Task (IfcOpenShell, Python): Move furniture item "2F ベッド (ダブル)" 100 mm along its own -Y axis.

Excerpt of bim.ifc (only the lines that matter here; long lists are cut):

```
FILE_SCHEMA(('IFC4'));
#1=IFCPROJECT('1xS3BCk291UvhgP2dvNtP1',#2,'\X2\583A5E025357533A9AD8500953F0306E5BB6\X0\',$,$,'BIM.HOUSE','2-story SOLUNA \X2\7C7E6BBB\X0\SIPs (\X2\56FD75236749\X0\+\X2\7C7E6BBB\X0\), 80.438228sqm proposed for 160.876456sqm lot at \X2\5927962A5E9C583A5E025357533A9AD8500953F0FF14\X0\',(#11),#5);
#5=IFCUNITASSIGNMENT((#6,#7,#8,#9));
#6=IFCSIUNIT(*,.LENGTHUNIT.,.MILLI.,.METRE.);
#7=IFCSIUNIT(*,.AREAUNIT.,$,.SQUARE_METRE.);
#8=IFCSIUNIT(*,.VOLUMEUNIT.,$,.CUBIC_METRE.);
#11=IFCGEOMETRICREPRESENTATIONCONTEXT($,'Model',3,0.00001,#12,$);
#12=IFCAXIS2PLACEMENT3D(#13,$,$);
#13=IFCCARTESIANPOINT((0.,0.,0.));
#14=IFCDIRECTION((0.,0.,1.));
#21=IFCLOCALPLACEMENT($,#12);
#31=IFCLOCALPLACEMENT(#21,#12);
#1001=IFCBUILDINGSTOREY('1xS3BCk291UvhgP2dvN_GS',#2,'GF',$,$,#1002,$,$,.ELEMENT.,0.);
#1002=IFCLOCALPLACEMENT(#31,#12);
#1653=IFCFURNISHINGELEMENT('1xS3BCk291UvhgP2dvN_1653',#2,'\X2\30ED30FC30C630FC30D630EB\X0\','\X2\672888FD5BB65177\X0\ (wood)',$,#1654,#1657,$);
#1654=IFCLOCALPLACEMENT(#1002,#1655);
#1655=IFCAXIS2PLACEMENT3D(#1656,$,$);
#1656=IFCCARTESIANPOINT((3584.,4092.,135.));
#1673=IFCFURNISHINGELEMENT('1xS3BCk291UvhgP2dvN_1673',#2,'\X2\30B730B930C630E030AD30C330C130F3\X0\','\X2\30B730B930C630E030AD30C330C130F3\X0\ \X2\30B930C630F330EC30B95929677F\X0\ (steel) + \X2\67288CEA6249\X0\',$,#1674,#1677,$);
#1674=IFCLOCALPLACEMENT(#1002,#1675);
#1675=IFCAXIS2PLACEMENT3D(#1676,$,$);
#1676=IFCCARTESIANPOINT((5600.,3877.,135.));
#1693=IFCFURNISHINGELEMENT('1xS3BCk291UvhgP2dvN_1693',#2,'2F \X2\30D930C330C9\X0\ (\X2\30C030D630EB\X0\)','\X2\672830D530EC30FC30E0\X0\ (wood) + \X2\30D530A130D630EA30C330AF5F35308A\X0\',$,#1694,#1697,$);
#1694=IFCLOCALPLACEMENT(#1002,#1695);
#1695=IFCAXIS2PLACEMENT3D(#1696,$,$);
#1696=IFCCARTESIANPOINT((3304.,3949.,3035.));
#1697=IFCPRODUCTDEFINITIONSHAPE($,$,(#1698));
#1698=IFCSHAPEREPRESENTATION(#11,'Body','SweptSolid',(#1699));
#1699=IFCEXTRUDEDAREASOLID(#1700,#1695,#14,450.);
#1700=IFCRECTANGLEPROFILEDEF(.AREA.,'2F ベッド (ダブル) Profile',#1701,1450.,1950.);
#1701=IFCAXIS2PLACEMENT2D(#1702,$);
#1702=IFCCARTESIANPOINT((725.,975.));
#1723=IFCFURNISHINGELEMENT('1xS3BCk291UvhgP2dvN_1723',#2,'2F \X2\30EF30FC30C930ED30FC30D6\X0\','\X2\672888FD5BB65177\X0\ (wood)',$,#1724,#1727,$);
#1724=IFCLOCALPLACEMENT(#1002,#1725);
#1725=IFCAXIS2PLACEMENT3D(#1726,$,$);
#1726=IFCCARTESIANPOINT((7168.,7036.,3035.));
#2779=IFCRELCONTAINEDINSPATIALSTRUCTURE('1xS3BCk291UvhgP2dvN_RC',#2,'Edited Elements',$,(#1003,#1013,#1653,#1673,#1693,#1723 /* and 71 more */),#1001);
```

```python
import ifcopenshell
import ifcopenshell.api.geometry
import ifcopenshell.util.placement

model = ifcopenshell.open("bim.ifc")

item = model.by_guid("1xS3BCk291UvhgP2dvN_1693")
matrix = ifcopenshell.util.placement.get_local_placement(item.ObjectPlacement)
matrix[:3, 3] -= matrix[:3, 1] * 100.0
ifcopenshell.api.geometry.edit_object_placement(model, product=item, matrix=matrix, is_si=False)

print(ifcopenshell.util.placement.get_local_placement(item.ObjectPlacement).round(3) + 0.0)

model.write("bim_updated.ifc")
```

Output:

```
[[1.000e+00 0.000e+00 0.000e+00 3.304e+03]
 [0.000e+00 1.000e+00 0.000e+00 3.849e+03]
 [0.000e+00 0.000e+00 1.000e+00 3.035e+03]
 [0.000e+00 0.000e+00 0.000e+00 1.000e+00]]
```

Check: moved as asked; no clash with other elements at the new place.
